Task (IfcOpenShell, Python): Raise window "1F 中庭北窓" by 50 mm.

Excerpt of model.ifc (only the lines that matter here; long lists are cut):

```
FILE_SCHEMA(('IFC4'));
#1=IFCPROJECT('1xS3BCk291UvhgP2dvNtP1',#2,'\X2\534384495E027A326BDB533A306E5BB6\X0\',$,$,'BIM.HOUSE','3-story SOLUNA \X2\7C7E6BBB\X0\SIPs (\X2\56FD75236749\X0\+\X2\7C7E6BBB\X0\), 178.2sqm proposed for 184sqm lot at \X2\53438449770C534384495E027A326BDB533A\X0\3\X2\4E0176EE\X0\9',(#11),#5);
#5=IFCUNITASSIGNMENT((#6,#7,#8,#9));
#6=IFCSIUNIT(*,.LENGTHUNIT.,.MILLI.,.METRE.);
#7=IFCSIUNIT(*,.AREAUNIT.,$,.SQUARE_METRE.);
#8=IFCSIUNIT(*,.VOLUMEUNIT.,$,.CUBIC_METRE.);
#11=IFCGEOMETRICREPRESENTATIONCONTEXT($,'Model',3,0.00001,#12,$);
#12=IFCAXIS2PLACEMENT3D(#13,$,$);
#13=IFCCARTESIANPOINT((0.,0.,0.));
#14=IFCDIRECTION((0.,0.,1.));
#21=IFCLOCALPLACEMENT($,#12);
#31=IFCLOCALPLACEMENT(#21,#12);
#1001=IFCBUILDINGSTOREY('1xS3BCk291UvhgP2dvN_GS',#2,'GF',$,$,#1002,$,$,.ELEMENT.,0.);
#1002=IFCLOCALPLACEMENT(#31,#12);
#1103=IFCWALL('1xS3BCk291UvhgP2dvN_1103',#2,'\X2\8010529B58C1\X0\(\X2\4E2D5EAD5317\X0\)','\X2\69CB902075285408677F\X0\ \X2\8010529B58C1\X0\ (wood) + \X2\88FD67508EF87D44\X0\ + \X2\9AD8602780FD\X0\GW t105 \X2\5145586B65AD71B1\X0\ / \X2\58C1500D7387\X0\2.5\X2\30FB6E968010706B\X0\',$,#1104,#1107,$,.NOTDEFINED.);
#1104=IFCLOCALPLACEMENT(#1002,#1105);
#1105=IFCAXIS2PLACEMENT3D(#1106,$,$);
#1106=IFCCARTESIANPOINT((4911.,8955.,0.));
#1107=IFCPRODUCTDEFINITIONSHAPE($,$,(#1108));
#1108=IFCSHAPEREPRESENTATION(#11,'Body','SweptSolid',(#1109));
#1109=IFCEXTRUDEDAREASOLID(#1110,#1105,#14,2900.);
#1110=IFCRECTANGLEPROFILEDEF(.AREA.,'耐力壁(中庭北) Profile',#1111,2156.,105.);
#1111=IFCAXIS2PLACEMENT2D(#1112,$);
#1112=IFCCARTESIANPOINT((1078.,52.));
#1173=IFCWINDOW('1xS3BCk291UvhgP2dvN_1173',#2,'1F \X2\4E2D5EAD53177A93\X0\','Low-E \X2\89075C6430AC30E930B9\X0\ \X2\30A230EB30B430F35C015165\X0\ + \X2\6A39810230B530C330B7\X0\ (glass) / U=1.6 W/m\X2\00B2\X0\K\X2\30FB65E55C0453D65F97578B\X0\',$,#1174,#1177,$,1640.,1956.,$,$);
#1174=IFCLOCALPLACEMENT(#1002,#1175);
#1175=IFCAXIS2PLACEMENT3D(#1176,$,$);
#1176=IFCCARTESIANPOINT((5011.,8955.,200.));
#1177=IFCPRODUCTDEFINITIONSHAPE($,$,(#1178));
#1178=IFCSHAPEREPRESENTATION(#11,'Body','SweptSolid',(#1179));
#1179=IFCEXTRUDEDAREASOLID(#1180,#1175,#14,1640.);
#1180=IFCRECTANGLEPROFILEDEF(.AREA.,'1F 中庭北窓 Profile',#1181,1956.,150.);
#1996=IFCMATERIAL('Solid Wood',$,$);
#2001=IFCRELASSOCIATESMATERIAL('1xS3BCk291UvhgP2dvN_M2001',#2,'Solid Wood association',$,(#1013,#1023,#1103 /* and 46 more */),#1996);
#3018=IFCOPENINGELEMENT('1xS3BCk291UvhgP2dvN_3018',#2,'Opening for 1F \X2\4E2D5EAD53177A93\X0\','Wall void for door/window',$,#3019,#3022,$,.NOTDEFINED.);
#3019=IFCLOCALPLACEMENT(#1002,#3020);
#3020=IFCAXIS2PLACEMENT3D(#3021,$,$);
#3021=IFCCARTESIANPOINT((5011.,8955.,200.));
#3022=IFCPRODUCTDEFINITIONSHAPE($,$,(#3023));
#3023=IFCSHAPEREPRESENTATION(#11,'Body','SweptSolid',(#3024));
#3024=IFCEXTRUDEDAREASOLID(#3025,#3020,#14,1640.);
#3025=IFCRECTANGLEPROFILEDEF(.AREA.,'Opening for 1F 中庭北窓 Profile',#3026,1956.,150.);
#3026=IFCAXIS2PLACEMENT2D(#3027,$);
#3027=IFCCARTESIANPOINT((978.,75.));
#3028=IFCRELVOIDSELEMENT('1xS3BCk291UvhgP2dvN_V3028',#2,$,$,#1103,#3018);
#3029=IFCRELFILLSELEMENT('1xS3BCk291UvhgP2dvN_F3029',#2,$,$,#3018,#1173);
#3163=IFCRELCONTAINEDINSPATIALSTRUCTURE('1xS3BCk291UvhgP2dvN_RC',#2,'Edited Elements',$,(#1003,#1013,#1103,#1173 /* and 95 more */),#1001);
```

```python
import numpy as np
import ifcopenshell
import ifcopenshell.api.geometry
import ifcopenshell.util.placement
import ifcopenshell.util.unit

model = ifcopenshell.open("model.ifc")
unit_scale = ifcopenshell.util.unit.calculate_unit_scale(model)

window = model.by_guid("1xS3BCk291UvhgP2dvN_1173")
opening = window.FillsVoids[0].RelatingOpeningElement
dz = 0.05 / unit_scale

shift = np.array([0.0, 0.0, dz])
# The window is not placed relative to its opening, so move both.
for product in (opening, window):
    matrix = ifcopenshell.util.placement.get_local_placement(product.ObjectPlacement)
    matrix[:3, 3] += shift
    ifcopenshell.api.geometry.edit_object_placement(model, product=product, matrix=matrix, is_si=False)

print(f"moved by {dz * unit_scale:+.3f} m")

model.write("model_v2.ifc")
```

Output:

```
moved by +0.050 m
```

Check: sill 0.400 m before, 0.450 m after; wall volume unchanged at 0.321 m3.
